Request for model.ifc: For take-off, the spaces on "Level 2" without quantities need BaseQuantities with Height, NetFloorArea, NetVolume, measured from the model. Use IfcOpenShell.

First a look at what the model holds.

```python
import ifcopenshell
import ifcopenshell.util.element
import ifcopenshell.util.unit

model = ifcopenshell.open("model.ifc")
print(model.schema)
for unit_type in ("LENGTHUNIT", "AREAUNIT", "VOLUMEUNIT"):
    print(unit_type, ifcopenshell.util.unit.calculate_unit_scale(model, unit_type))
storey = next(s for s in model.by_type("IfcBuildingStorey") if s.Name == "Level 2")
spaces = [e for e in ifcopenshell.util.element.get_decomposition(storey) if e.is_a("IfcSpace")]
for e in sorted(spaces, key=lambda e: e.id()):
    print(e.id(), e.is_a(), e.Name, list(ifcopenshell.util.element.get_psets(e, qtos_only=True)), sep=" | ")
```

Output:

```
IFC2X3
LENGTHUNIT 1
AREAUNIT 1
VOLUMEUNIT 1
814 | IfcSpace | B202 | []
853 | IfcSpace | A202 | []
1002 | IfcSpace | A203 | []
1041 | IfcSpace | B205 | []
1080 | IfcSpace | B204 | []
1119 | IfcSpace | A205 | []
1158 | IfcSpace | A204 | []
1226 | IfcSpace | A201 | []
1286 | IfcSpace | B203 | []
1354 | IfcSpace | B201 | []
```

```python
import ifcopenshell
import ifcopenshell.api.pset
import ifcopenshell.geom
import ifcopenshell.util.element
import ifcopenshell.util.shape
import ifcopenshell.util.unit

model = ifcopenshell.open("model.ifc")
unit_scale = ifcopenshell.util.unit.calculate_unit_scale(model)
area_scale = ifcopenshell.util.unit.calculate_unit_scale(model, "AREAUNIT")
volume_scale = ifcopenshell.util.unit.calculate_unit_scale(model, "VOLUMEUNIT")
settings = ifcopenshell.geom.settings()

storey = next(s for s in model.by_type("IfcBuildingStorey") if s.Name == "Level 2")
spaces = [e for e in ifcopenshell.util.element.get_decomposition(storey) if e.is_a("IfcSpace")]

for e in sorted(spaces, key=lambda e: e.id()):
    if ifcopenshell.util.element.get_psets(e, qtos_only=True, should_inherit=False):
        continue
    # Geometry comes back in metres, in the element's own axes.
    shape = ifcopenshell.geom.create_shape(settings, e)
    values = {
        "Height": ifcopenshell.util.shape.get_z(shape.geometry) / unit_scale,
        "NetFloorArea": ifcopenshell.util.shape.get_footprint_area(shape.geometry) / area_scale,
        "NetVolume": ifcopenshell.util.shape.get_volume(shape.geometry) / volume_scale,
    }
    qto = ifcopenshell.api.pset.add_qto(model, product=e, name="BaseQuantities")
    ifcopenshell.api.pset.edit_qto(model, qto=qto, properties=values)
    print(e.id(), {k: round(v, 3) for k, v in values.items()})

model.write("model-out.ifc")
```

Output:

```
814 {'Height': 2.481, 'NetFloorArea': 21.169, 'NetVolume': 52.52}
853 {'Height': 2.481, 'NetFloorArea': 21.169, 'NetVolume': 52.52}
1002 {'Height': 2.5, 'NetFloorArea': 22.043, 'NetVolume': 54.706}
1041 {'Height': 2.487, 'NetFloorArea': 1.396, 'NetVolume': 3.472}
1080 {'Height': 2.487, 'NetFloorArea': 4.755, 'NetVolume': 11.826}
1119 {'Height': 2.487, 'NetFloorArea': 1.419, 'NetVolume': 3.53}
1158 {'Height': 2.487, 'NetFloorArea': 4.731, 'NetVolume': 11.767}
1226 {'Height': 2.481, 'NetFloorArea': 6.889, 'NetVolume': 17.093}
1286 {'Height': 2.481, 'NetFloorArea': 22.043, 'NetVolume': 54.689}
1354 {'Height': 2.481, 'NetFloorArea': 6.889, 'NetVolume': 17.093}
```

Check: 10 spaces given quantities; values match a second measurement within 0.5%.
